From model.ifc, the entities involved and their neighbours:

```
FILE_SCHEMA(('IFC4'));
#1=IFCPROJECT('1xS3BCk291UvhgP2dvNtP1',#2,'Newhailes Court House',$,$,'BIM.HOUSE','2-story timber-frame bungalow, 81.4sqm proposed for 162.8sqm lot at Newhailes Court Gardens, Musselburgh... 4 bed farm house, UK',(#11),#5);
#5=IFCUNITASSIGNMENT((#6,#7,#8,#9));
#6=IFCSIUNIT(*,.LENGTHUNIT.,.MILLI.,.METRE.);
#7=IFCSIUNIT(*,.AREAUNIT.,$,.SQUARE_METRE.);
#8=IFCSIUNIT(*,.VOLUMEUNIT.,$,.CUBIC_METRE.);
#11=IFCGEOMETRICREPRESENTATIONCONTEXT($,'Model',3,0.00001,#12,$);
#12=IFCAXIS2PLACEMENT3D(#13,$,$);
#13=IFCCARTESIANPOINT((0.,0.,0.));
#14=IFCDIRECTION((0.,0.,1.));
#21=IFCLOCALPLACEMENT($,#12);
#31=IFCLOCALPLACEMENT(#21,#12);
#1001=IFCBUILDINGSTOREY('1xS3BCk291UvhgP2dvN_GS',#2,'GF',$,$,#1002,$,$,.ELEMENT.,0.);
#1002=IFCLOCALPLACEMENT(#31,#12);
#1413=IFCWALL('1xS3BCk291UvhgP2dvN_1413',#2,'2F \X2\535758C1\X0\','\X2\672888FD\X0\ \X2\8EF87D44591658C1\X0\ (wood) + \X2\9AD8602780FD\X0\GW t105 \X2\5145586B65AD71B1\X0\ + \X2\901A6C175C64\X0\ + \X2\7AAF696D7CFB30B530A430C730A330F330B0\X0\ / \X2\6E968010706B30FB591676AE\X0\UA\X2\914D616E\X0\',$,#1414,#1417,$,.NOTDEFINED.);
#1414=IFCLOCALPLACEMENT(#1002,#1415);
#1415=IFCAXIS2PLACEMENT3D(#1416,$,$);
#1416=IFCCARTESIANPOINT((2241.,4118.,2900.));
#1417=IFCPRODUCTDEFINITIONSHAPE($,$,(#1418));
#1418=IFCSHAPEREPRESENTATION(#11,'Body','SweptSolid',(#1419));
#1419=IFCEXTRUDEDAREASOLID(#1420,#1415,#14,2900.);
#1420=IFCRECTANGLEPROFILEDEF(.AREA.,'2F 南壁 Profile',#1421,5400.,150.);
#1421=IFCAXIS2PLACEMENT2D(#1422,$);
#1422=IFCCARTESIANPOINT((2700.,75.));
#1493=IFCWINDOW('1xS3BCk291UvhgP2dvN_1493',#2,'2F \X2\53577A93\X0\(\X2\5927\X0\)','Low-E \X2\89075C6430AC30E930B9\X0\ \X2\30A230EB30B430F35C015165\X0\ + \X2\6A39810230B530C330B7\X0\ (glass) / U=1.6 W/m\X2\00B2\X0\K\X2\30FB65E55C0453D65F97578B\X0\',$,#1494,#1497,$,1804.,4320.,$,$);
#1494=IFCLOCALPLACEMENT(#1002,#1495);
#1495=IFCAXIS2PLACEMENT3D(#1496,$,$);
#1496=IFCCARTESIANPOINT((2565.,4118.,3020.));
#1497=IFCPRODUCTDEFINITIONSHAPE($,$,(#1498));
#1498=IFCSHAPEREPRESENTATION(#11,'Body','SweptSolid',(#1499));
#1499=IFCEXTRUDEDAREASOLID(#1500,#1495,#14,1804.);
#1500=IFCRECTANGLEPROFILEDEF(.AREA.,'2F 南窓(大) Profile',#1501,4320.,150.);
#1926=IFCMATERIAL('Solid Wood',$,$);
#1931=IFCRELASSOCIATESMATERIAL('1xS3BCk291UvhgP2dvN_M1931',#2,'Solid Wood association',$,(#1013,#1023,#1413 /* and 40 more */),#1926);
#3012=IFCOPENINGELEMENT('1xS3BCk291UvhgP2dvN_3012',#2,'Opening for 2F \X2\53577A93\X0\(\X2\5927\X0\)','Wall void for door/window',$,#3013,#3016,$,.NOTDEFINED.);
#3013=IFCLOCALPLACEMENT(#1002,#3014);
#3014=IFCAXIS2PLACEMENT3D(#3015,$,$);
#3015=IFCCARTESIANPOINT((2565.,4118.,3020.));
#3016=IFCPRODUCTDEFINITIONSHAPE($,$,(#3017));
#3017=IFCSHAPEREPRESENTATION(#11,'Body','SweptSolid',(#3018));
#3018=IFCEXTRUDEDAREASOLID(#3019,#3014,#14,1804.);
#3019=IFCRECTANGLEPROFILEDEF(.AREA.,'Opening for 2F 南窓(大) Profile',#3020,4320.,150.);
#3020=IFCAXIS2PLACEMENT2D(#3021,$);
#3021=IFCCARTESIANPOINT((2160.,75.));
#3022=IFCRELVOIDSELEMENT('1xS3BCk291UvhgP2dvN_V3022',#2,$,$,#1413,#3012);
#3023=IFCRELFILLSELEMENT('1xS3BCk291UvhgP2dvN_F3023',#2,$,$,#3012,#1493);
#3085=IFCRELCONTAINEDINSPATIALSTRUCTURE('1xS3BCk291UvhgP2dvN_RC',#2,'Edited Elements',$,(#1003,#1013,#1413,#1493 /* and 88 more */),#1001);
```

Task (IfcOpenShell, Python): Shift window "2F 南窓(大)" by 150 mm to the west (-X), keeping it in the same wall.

```python
import ifcopenshell
import ifcopenshell.api.geometry
import ifcopenshell.util.placement
import ifcopenshell.util.unit

model = ifcopenshell.open("model.ifc")
unit_scale = ifcopenshell.util.unit.calculate_unit_scale(model)

window = model.by_id(1493)
opening = window.FillsVoids[0].RelatingOpeningElement
wall = opening.VoidsElements[0].RelatingBuildingElement

wall_matrix = ifcopenshell.util.placement.get_local_placement(wall.ObjectPlacement)
shift = wall_matrix[:3, 0] * -0.15 / unit_scale
before = ifcopenshell.util.placement.get_local_placement(window.ObjectPlacement)[:3, 3].copy()

# The window is not placed relative to its opening, so move both.
for product in (opening, window):
    matrix = ifcopenshell.util.placement.get_local_placement(product.ObjectPlacement)
    matrix[:3, 3] += shift
    ifcopenshell.api.geometry.edit_object_placement(model, product=product, matrix=matrix, is_si=False)

after = ifcopenshell.util.placement.get_local_placement(window.ObjectPlacement)[:3, 3]
print("window moved by", (after - before).round(3) + 0.0)

model.write("model_edited.ifc")
```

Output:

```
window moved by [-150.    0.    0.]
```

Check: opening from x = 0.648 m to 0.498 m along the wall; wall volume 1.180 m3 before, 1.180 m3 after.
